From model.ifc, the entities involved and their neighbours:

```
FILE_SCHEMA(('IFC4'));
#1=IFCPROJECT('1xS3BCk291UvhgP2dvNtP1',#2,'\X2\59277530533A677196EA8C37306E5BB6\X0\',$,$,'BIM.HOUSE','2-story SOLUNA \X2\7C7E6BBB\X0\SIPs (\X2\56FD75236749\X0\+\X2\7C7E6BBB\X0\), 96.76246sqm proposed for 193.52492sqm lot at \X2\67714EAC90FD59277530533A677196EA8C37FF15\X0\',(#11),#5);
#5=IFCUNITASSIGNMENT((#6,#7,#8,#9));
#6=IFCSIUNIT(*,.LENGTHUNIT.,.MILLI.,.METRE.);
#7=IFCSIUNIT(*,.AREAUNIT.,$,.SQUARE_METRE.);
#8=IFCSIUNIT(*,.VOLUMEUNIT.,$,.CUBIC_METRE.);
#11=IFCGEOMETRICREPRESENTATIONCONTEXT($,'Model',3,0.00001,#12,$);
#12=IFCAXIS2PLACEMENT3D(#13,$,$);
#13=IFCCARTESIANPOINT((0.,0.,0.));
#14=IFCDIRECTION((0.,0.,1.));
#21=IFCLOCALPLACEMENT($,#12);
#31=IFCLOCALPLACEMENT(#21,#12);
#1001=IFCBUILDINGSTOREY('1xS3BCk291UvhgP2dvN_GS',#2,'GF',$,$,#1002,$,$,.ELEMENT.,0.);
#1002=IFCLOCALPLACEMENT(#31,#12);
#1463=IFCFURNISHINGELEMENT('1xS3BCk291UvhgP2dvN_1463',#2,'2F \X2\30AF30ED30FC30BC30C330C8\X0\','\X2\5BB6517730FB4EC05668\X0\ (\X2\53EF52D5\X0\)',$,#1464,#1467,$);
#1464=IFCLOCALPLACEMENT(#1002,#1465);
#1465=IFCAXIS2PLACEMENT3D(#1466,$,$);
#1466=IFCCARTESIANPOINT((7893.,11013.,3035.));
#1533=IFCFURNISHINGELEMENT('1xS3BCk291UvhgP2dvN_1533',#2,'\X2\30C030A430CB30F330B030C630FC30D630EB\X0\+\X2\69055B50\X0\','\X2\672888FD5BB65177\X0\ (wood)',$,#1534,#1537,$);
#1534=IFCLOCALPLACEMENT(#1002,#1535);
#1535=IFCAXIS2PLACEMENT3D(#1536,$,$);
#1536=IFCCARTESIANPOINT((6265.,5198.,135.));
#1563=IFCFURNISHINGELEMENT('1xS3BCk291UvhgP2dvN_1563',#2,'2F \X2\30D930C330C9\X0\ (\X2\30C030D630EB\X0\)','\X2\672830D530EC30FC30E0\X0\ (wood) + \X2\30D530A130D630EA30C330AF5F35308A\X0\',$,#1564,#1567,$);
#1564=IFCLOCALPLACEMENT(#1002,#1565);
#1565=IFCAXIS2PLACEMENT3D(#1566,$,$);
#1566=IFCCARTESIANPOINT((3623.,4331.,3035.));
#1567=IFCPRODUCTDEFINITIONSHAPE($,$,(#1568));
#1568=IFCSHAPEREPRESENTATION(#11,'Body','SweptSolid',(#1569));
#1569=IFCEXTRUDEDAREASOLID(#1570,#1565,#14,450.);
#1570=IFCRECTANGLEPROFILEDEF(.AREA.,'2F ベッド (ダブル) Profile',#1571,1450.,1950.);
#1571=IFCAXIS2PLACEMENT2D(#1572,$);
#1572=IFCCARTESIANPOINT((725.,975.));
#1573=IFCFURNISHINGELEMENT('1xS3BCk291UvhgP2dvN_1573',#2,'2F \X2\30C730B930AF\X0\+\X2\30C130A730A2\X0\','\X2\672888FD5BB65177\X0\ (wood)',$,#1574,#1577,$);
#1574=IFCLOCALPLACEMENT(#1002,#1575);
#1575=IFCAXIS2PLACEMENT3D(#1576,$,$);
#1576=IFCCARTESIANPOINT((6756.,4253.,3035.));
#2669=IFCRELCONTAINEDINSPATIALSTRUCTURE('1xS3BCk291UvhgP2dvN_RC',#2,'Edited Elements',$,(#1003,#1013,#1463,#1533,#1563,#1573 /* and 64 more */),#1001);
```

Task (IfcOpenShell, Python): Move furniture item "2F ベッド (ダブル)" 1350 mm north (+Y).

```python
import ifcopenshell
import ifcopenshell.api.geometry
import ifcopenshell.util.placement
import ifcopenshell.util.unit

model = ifcopenshell.open("model.ifc")
unit_scale = ifcopenshell.util.unit.calculate_unit_scale(model)

item = model.by_id(1563)
matrix = ifcopenshell.util.placement.get_local_placement(item.ObjectPlacement)
matrix[1, 3] += 1.35 / unit_scale
ifcopenshell.api.geometry.edit_object_placement(model, product=item, matrix=matrix, is_si=False)

print(ifcopenshell.util.placement.get_local_placement(item.ObjectPlacement).round(3) + 0.0)

model.write("model_v2.ifc")
```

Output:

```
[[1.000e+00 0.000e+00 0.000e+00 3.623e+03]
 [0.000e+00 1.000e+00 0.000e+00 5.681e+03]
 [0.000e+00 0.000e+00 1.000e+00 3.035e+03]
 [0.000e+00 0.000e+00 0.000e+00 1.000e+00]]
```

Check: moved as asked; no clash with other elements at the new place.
